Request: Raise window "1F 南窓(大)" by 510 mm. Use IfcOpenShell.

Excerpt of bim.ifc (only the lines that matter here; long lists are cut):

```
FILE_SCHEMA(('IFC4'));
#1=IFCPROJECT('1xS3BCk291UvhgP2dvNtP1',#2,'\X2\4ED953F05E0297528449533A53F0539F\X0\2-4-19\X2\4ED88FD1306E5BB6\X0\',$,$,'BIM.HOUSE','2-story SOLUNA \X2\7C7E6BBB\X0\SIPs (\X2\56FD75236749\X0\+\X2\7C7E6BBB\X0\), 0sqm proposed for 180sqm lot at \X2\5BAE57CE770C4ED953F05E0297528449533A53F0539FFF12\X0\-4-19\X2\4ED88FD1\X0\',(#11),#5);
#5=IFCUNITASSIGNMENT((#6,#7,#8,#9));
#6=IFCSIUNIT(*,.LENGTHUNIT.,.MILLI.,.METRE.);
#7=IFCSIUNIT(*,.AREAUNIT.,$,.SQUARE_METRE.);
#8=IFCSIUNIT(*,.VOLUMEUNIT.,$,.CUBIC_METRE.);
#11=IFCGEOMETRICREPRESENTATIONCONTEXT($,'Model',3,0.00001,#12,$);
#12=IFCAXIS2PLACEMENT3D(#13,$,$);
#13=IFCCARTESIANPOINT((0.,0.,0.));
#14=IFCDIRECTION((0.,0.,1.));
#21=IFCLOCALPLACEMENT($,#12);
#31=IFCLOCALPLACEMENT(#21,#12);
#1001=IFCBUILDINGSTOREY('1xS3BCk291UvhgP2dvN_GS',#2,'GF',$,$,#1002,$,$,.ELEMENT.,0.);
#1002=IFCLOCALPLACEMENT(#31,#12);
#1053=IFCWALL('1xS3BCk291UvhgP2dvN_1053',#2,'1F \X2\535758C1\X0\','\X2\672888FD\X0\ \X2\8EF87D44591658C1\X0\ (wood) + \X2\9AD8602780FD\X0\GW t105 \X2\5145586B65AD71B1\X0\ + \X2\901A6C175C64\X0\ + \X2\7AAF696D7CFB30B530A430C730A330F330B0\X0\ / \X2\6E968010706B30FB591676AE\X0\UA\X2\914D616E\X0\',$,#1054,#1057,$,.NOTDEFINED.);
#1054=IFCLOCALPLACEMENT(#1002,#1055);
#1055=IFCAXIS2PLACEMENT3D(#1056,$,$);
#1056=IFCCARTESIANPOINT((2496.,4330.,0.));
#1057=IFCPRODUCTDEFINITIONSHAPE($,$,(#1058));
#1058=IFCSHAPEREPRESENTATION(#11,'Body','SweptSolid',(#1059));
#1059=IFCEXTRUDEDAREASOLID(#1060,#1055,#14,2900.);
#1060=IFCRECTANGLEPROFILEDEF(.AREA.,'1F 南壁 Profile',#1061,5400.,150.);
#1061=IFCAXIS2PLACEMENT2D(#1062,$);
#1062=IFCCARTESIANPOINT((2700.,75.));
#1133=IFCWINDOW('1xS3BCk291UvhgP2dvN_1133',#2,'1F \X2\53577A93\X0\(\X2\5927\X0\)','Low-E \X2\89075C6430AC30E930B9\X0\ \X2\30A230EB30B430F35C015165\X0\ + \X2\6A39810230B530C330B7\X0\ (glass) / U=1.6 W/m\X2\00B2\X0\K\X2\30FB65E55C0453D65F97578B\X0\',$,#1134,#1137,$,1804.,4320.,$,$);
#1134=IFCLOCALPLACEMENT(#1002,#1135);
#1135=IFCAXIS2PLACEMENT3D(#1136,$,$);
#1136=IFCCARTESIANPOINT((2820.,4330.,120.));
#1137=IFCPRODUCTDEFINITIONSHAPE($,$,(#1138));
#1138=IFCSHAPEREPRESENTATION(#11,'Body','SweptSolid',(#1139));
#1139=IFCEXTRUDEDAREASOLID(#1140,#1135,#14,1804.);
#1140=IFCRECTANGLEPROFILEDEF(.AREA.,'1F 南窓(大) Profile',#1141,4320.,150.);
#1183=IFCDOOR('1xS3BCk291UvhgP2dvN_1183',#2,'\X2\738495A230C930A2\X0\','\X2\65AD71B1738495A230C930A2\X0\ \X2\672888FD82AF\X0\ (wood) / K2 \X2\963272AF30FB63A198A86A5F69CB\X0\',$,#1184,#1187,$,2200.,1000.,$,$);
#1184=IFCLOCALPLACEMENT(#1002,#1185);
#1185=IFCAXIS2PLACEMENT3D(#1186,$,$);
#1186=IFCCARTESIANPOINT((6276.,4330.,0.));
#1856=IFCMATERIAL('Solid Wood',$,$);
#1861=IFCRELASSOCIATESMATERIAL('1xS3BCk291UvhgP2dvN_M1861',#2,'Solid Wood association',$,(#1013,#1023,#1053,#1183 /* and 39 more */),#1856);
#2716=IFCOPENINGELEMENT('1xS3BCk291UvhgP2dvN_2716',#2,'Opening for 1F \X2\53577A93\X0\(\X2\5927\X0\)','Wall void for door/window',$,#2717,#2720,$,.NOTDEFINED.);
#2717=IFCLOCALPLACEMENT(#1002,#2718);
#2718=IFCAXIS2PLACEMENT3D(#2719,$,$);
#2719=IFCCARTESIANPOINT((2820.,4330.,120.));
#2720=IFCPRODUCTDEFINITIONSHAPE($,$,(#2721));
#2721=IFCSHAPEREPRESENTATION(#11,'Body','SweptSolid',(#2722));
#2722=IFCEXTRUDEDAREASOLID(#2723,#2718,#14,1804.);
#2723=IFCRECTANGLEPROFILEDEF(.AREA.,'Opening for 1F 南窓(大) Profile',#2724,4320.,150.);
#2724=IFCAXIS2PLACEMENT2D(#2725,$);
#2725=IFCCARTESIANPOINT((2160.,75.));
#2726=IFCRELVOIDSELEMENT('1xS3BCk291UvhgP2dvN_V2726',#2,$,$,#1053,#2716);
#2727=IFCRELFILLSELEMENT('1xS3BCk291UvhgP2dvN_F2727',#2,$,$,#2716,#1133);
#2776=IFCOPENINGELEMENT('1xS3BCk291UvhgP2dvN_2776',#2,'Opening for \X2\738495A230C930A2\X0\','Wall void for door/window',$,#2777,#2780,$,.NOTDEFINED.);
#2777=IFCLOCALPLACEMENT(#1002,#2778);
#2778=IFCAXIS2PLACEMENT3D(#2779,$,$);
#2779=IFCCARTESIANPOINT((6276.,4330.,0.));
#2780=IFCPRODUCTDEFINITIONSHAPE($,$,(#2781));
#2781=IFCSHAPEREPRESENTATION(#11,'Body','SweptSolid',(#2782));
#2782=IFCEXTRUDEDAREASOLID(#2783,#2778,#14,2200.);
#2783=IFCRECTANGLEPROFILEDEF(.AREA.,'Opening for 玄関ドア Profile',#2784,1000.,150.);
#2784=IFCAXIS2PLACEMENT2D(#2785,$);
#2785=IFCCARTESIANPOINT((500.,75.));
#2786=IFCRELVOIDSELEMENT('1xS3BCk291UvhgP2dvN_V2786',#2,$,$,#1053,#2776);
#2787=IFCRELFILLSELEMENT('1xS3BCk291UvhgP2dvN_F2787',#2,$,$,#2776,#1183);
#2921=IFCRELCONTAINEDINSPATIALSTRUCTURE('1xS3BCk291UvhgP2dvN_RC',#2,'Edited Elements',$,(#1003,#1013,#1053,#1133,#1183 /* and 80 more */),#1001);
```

```python
import numpy as np
import ifcopenshell
import ifcopenshell.api.geometry
import ifcopenshell.util.placement
import ifcopenshell.util.unit

model = ifcopenshell.open("bim.ifc")
unit_scale = ifcopenshell.util.unit.calculate_unit_scale(model)

window = model.by_guid("1xS3BCk291UvhgP2dvN_1133")
opening = window.FillsVoids[0].RelatingOpeningElement
dz = 0.51 / unit_scale

shift = np.array([0.0, 0.0, dz])
# The window is not placed relative to its opening, so move both.
for product in (opening, window):
    matrix = ifcopenshell.util.placement.get_local_placement(product.ObjectPlacement)
    matrix[:3, 3] += shift
    ifcopenshell.api.geometry.edit_object_placement(model, product=product, matrix=matrix, is_si=False)

print(f"moved by {dz * unit_scale:+.3f} m")

model.write("bim_edited.ifc")
```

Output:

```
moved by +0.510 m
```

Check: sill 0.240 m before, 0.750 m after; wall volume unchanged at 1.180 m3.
